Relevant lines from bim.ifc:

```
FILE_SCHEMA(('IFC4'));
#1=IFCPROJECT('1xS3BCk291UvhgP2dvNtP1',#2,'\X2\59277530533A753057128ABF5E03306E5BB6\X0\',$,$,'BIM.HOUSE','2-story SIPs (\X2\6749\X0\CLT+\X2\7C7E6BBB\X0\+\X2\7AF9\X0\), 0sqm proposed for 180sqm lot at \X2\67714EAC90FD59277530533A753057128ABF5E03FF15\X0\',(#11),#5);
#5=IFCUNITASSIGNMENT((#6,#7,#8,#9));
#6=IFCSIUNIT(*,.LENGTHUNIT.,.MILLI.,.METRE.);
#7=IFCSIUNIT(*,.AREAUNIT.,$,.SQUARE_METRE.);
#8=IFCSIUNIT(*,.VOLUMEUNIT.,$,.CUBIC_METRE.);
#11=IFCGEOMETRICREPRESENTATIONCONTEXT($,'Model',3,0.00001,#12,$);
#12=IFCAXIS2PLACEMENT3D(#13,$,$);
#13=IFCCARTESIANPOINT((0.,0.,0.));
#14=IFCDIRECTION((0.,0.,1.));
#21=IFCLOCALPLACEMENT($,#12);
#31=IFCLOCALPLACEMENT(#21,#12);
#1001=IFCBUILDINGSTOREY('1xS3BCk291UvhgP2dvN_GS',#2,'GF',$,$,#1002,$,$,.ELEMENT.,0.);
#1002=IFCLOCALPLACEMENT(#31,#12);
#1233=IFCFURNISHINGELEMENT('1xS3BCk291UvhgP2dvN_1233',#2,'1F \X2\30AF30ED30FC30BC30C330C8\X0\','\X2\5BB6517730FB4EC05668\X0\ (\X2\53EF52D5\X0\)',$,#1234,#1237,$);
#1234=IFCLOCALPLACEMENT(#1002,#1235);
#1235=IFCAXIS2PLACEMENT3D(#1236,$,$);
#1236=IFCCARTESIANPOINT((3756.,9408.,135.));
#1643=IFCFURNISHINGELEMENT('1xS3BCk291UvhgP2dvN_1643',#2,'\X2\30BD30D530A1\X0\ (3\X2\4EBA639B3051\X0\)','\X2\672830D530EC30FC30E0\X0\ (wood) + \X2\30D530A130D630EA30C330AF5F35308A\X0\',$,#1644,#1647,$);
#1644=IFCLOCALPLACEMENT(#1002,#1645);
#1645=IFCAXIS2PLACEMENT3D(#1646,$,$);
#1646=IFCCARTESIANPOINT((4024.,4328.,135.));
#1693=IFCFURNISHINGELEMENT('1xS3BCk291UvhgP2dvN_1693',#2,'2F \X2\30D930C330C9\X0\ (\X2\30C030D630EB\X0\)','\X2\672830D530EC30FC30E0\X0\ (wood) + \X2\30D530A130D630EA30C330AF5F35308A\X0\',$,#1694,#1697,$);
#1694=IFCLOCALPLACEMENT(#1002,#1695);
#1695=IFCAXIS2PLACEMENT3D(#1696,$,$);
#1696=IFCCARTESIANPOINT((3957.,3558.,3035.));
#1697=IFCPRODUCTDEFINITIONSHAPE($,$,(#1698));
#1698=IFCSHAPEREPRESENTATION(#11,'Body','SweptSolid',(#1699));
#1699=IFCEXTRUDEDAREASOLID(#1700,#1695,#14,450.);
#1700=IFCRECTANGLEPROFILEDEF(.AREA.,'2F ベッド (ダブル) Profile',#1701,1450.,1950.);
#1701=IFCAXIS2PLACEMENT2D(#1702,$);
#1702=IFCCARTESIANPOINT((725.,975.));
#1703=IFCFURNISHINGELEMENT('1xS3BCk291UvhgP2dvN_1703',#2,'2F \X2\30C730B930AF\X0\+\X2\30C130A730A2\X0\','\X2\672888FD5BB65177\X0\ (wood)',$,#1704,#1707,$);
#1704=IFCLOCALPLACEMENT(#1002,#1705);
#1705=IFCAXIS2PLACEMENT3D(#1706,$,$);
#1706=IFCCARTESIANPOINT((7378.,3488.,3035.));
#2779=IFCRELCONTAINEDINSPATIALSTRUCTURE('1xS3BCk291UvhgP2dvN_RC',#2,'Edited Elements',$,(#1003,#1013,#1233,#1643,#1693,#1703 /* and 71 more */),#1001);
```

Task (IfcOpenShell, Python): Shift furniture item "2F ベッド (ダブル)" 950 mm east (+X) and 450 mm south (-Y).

```python
import ifcopenshell
import ifcopenshell.api.geometry
import ifcopenshell.util.placement
import ifcopenshell.util.unit

model = ifcopenshell.open("bim.ifc")
unit_scale = ifcopenshell.util.unit.calculate_unit_scale(model)

item = model.by_id(1693)
matrix = ifcopenshell.util.placement.get_local_placement(item.ObjectPlacement)
matrix[0, 3] += 0.95 / unit_scale
matrix[1, 3] -= 0.45 / unit_scale
ifcopenshell.api.geometry.edit_object_placement(model, product=item, matrix=matrix, is_si=False)

print(ifcopenshell.util.placement.get_local_placement(item.ObjectPlacement).round(3) + 0.0)

model.write("bim_v2.ifc")
```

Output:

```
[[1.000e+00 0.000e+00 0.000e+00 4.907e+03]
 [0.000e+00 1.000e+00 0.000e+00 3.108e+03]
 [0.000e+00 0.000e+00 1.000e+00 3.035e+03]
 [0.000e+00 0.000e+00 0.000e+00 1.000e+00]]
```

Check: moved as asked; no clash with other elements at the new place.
